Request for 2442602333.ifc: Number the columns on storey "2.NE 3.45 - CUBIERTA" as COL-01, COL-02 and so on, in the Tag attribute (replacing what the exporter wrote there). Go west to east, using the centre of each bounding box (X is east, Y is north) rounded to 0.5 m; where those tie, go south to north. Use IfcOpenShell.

First a look at what the model holds.

```python
import ifcopenshell
import ifcopenshell.util.element
import ifcopenshell.util.placement

model = ifcopenshell.open("2442602333.ifc")
print(model.schema)
storey = next(s for s in model.by_type("IfcBuildingStorey") if s.Name == "2.NE 3.45 - CUBIERTA")
columns = [e for e in ifcopenshell.util.element.get_decomposition(storey) if e.is_a("IfcColumn")]
for e in sorted(columns, key=lambda e: e.id()):
    origin = ifcopenshell.util.placement.get_local_placement(e.ObjectPlacement)[:3, 3]
    print(e.id(), e.Tag, e.Name, origin.round(2) + 0.0, sep=" | ")
```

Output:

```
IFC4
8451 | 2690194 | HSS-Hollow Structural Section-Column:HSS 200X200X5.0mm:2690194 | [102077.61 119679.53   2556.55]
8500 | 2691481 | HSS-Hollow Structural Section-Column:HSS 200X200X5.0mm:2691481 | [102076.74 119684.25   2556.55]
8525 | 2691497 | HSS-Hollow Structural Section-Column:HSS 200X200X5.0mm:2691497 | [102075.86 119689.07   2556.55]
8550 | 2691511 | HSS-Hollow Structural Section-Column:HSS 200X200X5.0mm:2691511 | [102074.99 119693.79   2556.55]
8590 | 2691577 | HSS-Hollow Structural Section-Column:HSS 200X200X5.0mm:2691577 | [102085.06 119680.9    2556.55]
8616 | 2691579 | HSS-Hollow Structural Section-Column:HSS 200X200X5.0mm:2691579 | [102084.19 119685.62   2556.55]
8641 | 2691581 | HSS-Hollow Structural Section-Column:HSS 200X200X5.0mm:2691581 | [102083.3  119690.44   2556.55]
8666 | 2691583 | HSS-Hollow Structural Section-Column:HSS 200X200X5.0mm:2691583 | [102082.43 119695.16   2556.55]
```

```python
import ifcopenshell
import ifcopenshell.geom
import ifcopenshell.util.element
import ifcopenshell.util.shape

model = ifcopenshell.open("2442602333.ifc")
settings = ifcopenshell.geom.settings()
settings.set("use-world-coords", True)


def centre(element):
    shape = ifcopenshell.geom.create_shape(settings, element)
    return ifcopenshell.util.shape.get_bbox_centroid(shape.geometry)


storey = next(s for s in model.by_type("IfcBuildingStorey") if s.Name == "2.NE 3.45 - CUBIERTA")
columns = [e for e in ifcopenshell.util.element.get_decomposition(storey) if e.is_a("IfcColumn")]

# Insertion points can sit at a corner or the storey origin, so sort by the geometry (in metres).
centres = {e: centre(e) for e in columns}
columns.sort(key=lambda e: (round(centres[e][0] / 0.5), centres[e][1]))

for i, e in enumerate(columns, start=1):
    number = f"COL-{i:02d}"
    e.Tag = number
    print(e.id(), number)

model.write("2442602333_rev.ifc")
```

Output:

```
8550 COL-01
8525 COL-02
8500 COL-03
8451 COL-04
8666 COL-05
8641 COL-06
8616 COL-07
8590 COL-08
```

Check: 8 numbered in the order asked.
